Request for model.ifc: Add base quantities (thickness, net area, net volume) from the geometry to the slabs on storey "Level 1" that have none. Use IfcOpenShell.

First a look at what the model holds.

```python
import ifcopenshell
import ifcopenshell.util.element
import ifcopenshell.util.unit

model = ifcopenshell.open("model.ifc")
print(model.schema)
for unit_type in ("LENGTHUNIT", "AREAUNIT", "VOLUMEUNIT"):
    print(unit_type, ifcopenshell.util.unit.calculate_unit_scale(model, unit_type))
storey = next(s for s in model.by_type("IfcBuildingStorey") if s.Name == "Level 1")
slabs = [e for e in ifcopenshell.util.element.get_decomposition(storey) if e.is_a("IfcSlab")]
for e in sorted(slabs, key=lambda e: e.id()):
    print(e.id(), e.is_a(), e.Name, list(ifcopenshell.util.element.get_psets(e, qtos_only=True)), sep=" | ")
```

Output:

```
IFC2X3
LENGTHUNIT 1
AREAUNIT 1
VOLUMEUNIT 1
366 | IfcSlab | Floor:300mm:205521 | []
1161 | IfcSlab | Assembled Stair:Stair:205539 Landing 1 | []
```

```python
import ifcopenshell
import ifcopenshell.api.pset
import ifcopenshell.geom
import ifcopenshell.util.element
import ifcopenshell.util.shape
import ifcopenshell.util.unit

model = ifcopenshell.open("model.ifc")
unit_scale = ifcopenshell.util.unit.calculate_unit_scale(model)
area_scale = ifcopenshell.util.unit.calculate_unit_scale(model, "AREAUNIT")
volume_scale = ifcopenshell.util.unit.calculate_unit_scale(model, "VOLUMEUNIT")
settings = ifcopenshell.geom.settings()

storey = next(s for s in model.by_type("IfcBuildingStorey") if s.Name == "Level 1")
slabs = [e for e in ifcopenshell.util.element.get_decomposition(storey) if e.is_a("IfcSlab")]

for e in sorted(slabs, key=lambda e: e.id()):
    if ifcopenshell.util.element.get_psets(e, qtos_only=True, should_inherit=False):
        continue
    # Geometry comes back in metres, in the element's own axes.
    shape = ifcopenshell.geom.create_shape(settings, e)
    values = {
        "Width": ifcopenshell.util.shape.get_z(shape.geometry) / unit_scale,
        "NetArea": ifcopenshell.util.shape.get_footprint_area(shape.geometry) / area_scale,
        "NetVolume": ifcopenshell.util.shape.get_volume(shape.geometry) / volume_scale,
    }
    qto = ifcopenshell.api.pset.add_qto(model, product=e, name="BaseQuantities")
    ifcopenshell.api.pset.edit_qto(model, qto=qto, properties=values)
    print(e.id(), {k: round(v, 3) for k, v in values.items()})

model.write("model-out.ifc")
```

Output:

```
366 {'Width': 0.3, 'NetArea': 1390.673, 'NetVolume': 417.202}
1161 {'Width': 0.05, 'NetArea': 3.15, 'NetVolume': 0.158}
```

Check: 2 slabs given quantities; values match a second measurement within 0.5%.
